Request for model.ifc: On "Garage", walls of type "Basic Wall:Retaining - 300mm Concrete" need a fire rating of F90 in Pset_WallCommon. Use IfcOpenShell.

First a look at what the model holds.

```python
import ifcopenshell
import ifcopenshell.util.element

model = ifcopenshell.open("model.ifc")
print(model.schema)
storey = next(s for s in model.by_type("IfcBuildingStorey") if s.Name == "Garage")
walls = [e for e in ifcopenshell.util.element.get_decomposition(storey) if e.is_a("IfcWall")]
seen = {}
for e in walls:
    element_type = ifcopenshell.util.element.get_type(e)
    key = (element_type.Name if element_type != e and element_type else None, ifcopenshell.util.element.get_pset(e, "Pset_WallCommon", "FireRating"))
    seen[key] = seen.get(key, 0) + 1
for (name, value), count in sorted(seen.items(), key=str):
    print(count, "x", name, "|", value)
```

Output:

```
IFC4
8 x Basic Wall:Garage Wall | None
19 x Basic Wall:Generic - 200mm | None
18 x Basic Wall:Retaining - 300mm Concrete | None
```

```python
import ifcopenshell
import ifcopenshell.api.pset
import ifcopenshell.util.element

model = ifcopenshell.open("model.ifc")

storey = next(s for s in model.by_type("IfcBuildingStorey") if s.Name == "Garage")
walls = [e for e in ifcopenshell.util.element.get_decomposition(storey) if e.is_a("IfcWall")]

count = 0
for e in walls:
    element_type = ifcopenshell.util.element.get_type(e)
    if element_type in (None, e) or element_type.Name != "Basic Wall:Retaining - 300mm Concrete":
        continue
    # add_pset returns the element's existing set when there is one.
    pset = ifcopenshell.api.pset.add_pset(model, product=e, name="Pset_WallCommon")
    ifcopenshell.api.pset.edit_pset(model, pset=pset, properties={"FireRating": "F90"})
    count += 1

print(count, "walls updated")

model.write("model_edited.ifc")
```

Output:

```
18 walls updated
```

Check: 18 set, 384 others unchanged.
